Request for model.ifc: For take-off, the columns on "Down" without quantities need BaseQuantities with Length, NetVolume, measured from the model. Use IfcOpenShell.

First a look at what the model holds.

```python
import ifcopenshell
import ifcopenshell.util.element
import ifcopenshell.util.unit

model = ifcopenshell.open("model.ifc")
print(model.schema)
for unit_type in ("LENGTHUNIT", "AREAUNIT", "VOLUMEUNIT"):
    print(unit_type, ifcopenshell.util.unit.calculate_unit_scale(model, unit_type))
storey = next(s for s in model.by_type("IfcBuildingStorey") if s.Name == "Down")
columns = [e for e in ifcopenshell.util.element.get_decomposition(storey) if e.is_a("IfcColumn")]
for e in sorted(columns, key=lambda e: e.id()):
    print(e.id(), e.is_a(), e.Name, list(ifcopenshell.util.element.get_psets(e, qtos_only=True)), sep=" | ")
```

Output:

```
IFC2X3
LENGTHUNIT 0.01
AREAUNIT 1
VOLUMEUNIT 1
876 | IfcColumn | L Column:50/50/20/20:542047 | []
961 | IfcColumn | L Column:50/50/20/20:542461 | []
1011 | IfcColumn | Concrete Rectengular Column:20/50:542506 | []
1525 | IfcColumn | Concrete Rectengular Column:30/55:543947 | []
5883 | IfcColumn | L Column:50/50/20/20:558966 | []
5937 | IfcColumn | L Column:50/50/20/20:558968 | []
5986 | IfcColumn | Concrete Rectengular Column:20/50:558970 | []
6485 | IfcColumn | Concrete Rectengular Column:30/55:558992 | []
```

```python
import ifcopenshell
import ifcopenshell.api.pset
import ifcopenshell.geom
import ifcopenshell.util.element
import ifcopenshell.util.shape
import ifcopenshell.util.unit

model = ifcopenshell.open("model.ifc")
unit_scale = ifcopenshell.util.unit.calculate_unit_scale(model)
volume_scale = ifcopenshell.util.unit.calculate_unit_scale(model, "VOLUMEUNIT")
settings = ifcopenshell.geom.settings()

storey = next(s for s in model.by_type("IfcBuildingStorey") if s.Name == "Down")
columns = [e for e in ifcopenshell.util.element.get_decomposition(storey) if e.is_a("IfcColumn")]

for e in sorted(columns, key=lambda e: e.id()):
    if ifcopenshell.util.element.get_psets(e, qtos_only=True, should_inherit=False):
        continue
    # Geometry comes back in metres, in the element's own axes.
    shape = ifcopenshell.geom.create_shape(settings, e)
    values = {
        "Length": ifcopenshell.util.shape.get_z(shape.geometry) / unit_scale,
        "NetVolume": ifcopenshell.util.shape.get_volume(shape.geometry) / volume_scale,
    }
    qto = ifcopenshell.api.pset.add_qto(model, product=e, name="BaseQuantities")
    ifcopenshell.api.pset.edit_qto(model, qto=qto, properties=values)
    print(e.id(), {k: round(v, 3) for k, v in values.items()})

model.write("model_v2.ifc")
```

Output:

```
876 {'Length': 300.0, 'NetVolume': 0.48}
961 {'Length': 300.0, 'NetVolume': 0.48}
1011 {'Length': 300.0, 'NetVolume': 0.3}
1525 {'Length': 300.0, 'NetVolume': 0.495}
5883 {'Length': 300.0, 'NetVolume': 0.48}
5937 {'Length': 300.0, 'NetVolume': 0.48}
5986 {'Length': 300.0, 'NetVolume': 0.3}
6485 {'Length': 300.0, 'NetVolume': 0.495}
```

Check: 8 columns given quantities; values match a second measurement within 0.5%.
